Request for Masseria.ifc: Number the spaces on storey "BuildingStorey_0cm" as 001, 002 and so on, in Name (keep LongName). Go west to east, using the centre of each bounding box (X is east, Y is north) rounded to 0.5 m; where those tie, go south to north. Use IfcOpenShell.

First a look at what the model holds.

```python
import ifcopenshell
import ifcopenshell.util.element
import ifcopenshell.util.placement

model = ifcopenshell.open("Masseria.ifc")
print(model.schema)
storey = next(s for s in model.by_type("IfcBuildingStorey") if s.Name == "BuildingStorey_0cm")
spaces = [e for e in ifcopenshell.util.element.get_decomposition(storey) if e.is_a("IfcSpace")]
for e in sorted(spaces, key=lambda e: e.id()):
    origin = ifcopenshell.util.placement.get_local_placement(e.ObjectPlacement)[:3, 3]
    print(e.id(), e.Name, e.LongName, origin.round(2) + 0.0, sep=" | ")
```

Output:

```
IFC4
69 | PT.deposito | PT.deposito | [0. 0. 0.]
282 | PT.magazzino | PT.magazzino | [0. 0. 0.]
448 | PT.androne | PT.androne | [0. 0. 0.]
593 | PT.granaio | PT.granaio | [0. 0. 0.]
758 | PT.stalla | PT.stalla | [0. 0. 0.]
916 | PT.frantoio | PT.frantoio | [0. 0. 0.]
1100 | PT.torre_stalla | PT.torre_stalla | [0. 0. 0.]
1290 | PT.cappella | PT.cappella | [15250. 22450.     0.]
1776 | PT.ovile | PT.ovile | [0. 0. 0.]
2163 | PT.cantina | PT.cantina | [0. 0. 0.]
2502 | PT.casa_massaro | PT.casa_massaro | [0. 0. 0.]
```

```python
import ifcopenshell
import ifcopenshell.geom
import ifcopenshell.util.element
import ifcopenshell.util.shape

model = ifcopenshell.open("Masseria.ifc")
settings = ifcopenshell.geom.settings()
settings.set("use-world-coords", True)


def centre(element):
    shape = ifcopenshell.geom.create_shape(settings, element)
    return ifcopenshell.util.shape.get_bbox_centroid(shape.geometry)


storey = next(s for s in model.by_type("IfcBuildingStorey") if s.Name == "BuildingStorey_0cm")
spaces = [e for e in ifcopenshell.util.element.get_decomposition(storey) if e.is_a("IfcSpace")]

# Insertion points can sit at a corner or the storey origin, so sort by the geometry (in metres).
centres = {e: centre(e) for e in spaces}
spaces.sort(key=lambda e: (round(centres[e][0] / 0.5), centres[e][1]))

for i, e in enumerate(spaces, start=1):
    number = f"0{i:02d}"
    e.Name = number
    print(e.id(), number)

model.write("Masseria-out.ifc")
```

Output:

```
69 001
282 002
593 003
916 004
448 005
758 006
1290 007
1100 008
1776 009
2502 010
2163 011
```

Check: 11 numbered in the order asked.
